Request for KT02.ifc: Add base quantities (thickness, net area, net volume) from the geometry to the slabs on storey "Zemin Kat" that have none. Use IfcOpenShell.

First a look at what the model holds.

```python
import ifcopenshell
import ifcopenshell.util.element
import ifcopenshell.util.unit

model = ifcopenshell.open("KT02.ifc")
print(model.schema)
for unit_type in ("LENGTHUNIT", "AREAUNIT", "VOLUMEUNIT"):
    print(unit_type, ifcopenshell.util.unit.calculate_unit_scale(model, unit_type))
storey = next(s for s in model.by_type("IfcBuildingStorey") if s.Name == "Zemin Kat")
slabs = [e for e in ifcopenshell.util.element.get_decomposition(storey) if e.is_a("IfcSlab")]
for e in sorted(slabs, key=lambda e: e.id()):
    print(e.id(), e.is_a(), e.Name, list(ifcopenshell.util.element.get_psets(e, qtos_only=True)), sep=" | ")
```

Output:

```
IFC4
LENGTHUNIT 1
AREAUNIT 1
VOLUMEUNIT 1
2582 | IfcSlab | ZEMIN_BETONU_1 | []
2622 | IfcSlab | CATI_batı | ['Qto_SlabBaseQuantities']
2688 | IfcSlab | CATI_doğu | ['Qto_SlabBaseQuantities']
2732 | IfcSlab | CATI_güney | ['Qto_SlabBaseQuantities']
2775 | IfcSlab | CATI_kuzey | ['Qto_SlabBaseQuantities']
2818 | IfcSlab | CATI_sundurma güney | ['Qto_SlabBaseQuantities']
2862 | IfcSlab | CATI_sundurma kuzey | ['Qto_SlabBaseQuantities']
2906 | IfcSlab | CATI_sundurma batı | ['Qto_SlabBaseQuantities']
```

```python
import ifcopenshell
import ifcopenshell.api.pset
import ifcopenshell.geom
import ifcopenshell.util.element
import ifcopenshell.util.shape
import ifcopenshell.util.unit

model = ifcopenshell.open("KT02.ifc")
unit_scale = ifcopenshell.util.unit.calculate_unit_scale(model)
area_scale = ifcopenshell.util.unit.calculate_unit_scale(model, "AREAUNIT")
volume_scale = ifcopenshell.util.unit.calculate_unit_scale(model, "VOLUMEUNIT")
settings = ifcopenshell.geom.settings()

storey = next(s for s in model.by_type("IfcBuildingStorey") if s.Name == "Zemin Kat")
slabs = [e for e in ifcopenshell.util.element.get_decomposition(storey) if e.is_a("IfcSlab")]

for e in sorted(slabs, key=lambda e: e.id()):
    if ifcopenshell.util.element.get_psets(e, qtos_only=True, should_inherit=False):
        continue
    # Geometry comes back in metres, in the element's own axes.
    shape = ifcopenshell.geom.create_shape(settings, e)
    values = {
        "Width": ifcopenshell.util.shape.get_z(shape.geometry) / unit_scale,
        "NetArea": ifcopenshell.util.shape.get_footprint_area(shape.geometry) / area_scale,
        "NetVolume": ifcopenshell.util.shape.get_volume(shape.geometry) / volume_scale,
    }
    qto = ifcopenshell.api.pset.add_qto(model, product=e, name="Qto_SlabBaseQuantities")
    ifcopenshell.api.pset.edit_qto(model, qto=qto, properties=values)
    print(e.id(), {k: round(v, 3) for k, v in values.items()})

model.write("KT02_v2.ifc")
```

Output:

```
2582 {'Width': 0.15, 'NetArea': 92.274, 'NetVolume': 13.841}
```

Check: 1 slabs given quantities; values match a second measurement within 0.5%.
